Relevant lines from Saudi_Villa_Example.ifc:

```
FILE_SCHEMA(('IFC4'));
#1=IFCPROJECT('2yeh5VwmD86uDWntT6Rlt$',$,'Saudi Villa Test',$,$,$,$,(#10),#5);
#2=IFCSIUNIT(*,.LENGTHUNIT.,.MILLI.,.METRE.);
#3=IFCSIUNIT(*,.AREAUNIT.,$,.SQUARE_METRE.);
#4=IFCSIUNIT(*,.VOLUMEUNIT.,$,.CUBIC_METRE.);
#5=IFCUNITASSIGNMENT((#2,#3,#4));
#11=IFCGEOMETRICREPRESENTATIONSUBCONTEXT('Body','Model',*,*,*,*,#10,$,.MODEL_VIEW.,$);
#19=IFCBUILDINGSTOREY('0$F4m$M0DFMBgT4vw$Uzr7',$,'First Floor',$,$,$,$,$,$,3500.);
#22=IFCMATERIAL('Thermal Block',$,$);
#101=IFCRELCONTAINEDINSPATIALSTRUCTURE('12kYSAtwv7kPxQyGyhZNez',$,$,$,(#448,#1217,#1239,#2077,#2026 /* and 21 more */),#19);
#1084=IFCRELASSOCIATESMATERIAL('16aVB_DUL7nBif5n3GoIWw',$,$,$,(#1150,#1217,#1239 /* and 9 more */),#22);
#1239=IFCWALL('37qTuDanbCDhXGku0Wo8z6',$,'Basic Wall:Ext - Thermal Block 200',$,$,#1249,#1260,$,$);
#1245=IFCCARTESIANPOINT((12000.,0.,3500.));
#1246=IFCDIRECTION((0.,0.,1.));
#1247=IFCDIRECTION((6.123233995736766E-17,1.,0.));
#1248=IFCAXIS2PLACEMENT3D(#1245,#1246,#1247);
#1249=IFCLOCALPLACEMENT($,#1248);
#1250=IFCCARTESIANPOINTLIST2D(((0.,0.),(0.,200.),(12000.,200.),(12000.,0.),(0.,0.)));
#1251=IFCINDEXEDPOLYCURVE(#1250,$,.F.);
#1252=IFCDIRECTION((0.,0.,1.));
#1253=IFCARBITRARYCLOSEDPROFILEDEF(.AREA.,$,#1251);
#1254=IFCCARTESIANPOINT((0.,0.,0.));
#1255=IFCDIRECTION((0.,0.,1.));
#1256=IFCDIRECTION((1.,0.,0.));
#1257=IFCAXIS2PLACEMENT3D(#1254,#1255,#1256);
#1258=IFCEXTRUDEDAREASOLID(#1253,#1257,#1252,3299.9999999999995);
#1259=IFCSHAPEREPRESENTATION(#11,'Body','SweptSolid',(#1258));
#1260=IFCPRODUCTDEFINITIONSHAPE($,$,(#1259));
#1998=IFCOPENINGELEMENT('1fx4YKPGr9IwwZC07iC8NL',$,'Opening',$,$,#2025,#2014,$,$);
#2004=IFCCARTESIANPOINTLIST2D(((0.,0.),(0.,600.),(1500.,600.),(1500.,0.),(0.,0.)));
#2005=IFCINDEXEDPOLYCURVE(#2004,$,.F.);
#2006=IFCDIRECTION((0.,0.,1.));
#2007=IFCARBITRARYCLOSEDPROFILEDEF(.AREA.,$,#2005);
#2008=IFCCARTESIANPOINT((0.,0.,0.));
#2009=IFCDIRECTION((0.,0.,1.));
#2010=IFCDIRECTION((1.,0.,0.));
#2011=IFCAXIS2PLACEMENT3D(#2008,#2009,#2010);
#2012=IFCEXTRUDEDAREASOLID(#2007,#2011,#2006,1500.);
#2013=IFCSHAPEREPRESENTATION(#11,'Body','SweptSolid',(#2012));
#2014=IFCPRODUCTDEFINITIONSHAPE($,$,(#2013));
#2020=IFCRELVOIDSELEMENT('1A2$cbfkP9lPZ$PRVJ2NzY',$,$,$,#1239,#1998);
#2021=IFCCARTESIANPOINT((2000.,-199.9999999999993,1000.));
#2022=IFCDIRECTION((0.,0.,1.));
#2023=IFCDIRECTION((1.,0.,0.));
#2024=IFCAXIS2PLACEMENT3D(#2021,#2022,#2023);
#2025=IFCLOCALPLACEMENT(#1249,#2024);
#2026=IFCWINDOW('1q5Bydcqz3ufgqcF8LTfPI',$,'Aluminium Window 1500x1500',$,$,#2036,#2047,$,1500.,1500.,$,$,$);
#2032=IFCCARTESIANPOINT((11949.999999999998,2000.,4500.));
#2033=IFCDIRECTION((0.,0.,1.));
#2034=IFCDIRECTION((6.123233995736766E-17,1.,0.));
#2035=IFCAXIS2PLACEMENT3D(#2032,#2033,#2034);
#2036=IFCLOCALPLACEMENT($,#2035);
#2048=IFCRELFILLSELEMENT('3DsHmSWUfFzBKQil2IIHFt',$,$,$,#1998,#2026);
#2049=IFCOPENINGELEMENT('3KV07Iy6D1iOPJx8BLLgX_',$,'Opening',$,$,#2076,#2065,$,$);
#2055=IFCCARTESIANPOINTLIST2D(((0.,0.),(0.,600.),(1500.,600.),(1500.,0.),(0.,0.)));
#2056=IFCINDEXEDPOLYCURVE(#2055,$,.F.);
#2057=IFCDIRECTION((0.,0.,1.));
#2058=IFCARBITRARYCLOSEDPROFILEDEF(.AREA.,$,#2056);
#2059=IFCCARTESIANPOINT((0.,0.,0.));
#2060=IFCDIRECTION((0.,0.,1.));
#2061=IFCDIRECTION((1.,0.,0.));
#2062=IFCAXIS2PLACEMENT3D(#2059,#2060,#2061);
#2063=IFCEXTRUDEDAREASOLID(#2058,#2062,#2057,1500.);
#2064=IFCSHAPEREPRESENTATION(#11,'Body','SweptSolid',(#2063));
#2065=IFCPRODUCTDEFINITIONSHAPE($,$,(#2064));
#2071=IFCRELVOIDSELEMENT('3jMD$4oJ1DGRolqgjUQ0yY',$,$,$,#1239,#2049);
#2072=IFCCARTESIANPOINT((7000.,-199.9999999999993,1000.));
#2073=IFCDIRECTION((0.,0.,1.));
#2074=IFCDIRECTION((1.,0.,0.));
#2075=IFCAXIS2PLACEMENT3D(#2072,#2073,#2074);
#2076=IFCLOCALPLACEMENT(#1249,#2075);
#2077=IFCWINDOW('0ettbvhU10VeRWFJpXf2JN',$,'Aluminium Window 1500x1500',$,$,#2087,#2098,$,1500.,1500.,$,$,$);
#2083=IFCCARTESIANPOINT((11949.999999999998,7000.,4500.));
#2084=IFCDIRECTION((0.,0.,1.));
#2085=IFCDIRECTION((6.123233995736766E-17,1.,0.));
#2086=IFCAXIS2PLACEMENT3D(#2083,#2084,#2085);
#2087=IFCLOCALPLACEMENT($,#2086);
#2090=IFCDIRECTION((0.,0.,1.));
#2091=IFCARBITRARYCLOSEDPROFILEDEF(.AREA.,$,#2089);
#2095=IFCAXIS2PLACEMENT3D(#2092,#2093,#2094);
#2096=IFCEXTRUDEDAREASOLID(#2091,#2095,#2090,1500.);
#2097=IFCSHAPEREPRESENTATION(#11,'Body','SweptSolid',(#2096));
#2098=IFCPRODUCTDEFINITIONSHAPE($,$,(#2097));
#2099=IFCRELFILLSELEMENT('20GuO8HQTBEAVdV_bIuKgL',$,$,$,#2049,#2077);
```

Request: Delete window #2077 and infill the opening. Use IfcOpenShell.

```python
import ifcopenshell
import ifcopenshell.api.feature
import ifcopenshell.api.root
import ifcopenshell.geom
import ifcopenshell.util.shape

model = ifcopenshell.open("Saudi_Villa_Example.ifc")
settings = ifcopenshell.geom.settings()


def volume(element):
    """Net volume in cubic metres, openings subtracted."""
    shape = ifcopenshell.geom.create_shape(settings, element)
    return ifcopenshell.util.shape.get_volume(shape.geometry)


window = model.by_id(2077)
opening = window.FillsVoids[0].RelatingOpeningElement
wall = opening.VoidsElements[0].RelatingBuildingElement
before = volume(wall)

ifcopenshell.api.root.remove_product(model, product=window)
ifcopenshell.api.feature.remove_feature(model, feature=opening)

after = volume(wall)

print(f"wall volume {before:.3f} -> {after:.3f} m3")

model.write("Saudi_Villa_Example-out.ifc")
```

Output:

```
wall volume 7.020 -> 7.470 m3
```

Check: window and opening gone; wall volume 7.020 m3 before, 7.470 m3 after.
